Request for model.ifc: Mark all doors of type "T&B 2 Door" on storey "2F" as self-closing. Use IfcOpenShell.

First a look at what the model holds.

```python
import ifcopenshell
import ifcopenshell.util.element

model = ifcopenshell.open("model.ifc")
print(model.schema)
storey = next(s for s in model.by_type("IfcBuildingStorey") if s.Name == "2F")
doors = [e for e in ifcopenshell.util.element.get_decomposition(storey) if e.is_a("IfcDoor")]
seen = {}
for e in doors:
    element_type = ifcopenshell.util.element.get_type(e)
    key = (element_type.Name if element_type != e and element_type else None, ifcopenshell.util.element.get_pset(e, "Pset_DoorCommon", "SelfClosing"))
    seen[key] = seen.get(key, 0) + 1
for (name, value), count in sorted(seen.items(), key=str):
    print(count, "x", name, "|", value)
```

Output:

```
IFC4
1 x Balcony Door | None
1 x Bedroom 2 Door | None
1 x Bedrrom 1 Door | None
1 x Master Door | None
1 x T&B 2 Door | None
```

```python
import ifcopenshell
import ifcopenshell.api.pset
import ifcopenshell.util.element

model = ifcopenshell.open("model.ifc")

storey = next(s for s in model.by_type("IfcBuildingStorey") if s.Name == "2F")
doors = [e for e in ifcopenshell.util.element.get_decomposition(storey) if e.is_a("IfcDoor")]

count = 0
for e in doors:
    element_type = ifcopenshell.util.element.get_type(e)
    if element_type in (None, e) or element_type.Name != "T&B 2 Door":
        continue
    # add_pset returns the element's existing set when there is one.
    pset = ifcopenshell.api.pset.add_pset(model, product=e, name="Pset_DoorCommon")
    ifcopenshell.api.pset.edit_pset(model, pset=pset, properties={"SelfClosing": True})
    count += 1

print(count, "doors updated")

model.write("model_updated.ifc")
```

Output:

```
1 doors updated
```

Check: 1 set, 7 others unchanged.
